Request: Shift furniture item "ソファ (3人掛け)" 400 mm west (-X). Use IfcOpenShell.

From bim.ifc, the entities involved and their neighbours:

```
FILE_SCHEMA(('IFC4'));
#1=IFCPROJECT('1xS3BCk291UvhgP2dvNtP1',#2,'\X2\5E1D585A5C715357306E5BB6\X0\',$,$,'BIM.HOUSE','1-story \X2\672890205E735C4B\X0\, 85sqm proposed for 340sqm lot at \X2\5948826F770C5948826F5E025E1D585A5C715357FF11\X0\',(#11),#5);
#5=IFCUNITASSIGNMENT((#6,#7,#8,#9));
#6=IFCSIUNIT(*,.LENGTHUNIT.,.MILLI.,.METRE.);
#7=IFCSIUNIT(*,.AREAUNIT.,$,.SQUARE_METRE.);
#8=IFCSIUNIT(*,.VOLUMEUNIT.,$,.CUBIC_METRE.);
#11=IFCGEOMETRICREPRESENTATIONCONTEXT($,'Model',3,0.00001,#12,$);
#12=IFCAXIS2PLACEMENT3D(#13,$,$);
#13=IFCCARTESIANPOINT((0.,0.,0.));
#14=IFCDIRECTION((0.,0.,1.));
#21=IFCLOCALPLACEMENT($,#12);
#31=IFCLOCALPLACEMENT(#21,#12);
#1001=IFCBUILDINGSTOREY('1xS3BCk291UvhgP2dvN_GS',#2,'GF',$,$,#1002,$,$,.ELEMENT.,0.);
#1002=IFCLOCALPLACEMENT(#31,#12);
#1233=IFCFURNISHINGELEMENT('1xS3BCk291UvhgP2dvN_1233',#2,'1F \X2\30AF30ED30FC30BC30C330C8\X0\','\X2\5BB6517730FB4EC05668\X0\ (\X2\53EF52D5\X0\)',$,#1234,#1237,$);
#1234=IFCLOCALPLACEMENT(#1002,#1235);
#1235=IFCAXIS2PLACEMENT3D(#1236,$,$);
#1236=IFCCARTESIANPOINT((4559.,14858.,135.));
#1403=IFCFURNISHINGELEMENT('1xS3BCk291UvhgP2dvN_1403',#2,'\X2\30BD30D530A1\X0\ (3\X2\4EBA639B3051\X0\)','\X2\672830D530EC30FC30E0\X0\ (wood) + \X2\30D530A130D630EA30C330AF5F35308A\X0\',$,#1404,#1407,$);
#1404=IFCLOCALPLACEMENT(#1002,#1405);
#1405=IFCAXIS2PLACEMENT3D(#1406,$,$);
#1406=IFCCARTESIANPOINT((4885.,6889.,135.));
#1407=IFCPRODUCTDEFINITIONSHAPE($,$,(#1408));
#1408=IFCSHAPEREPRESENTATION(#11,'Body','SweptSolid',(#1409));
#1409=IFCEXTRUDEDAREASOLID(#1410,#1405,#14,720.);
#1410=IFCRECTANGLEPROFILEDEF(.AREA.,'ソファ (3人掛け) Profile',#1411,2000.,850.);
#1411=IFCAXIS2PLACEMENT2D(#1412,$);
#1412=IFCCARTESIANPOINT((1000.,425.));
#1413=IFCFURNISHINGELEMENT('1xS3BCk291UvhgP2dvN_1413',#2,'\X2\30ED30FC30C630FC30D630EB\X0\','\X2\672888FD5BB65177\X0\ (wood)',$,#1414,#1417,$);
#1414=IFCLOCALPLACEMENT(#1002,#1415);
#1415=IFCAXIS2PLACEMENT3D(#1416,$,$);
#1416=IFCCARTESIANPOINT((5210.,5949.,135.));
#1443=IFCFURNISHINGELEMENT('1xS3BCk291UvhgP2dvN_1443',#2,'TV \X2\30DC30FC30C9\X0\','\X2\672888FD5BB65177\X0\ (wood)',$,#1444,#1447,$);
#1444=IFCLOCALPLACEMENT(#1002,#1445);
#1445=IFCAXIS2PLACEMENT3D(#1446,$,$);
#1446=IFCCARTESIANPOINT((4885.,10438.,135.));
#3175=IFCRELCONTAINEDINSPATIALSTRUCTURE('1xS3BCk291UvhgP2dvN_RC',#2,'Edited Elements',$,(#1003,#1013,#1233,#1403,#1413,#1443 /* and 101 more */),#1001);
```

```python
import ifcopenshell
import ifcopenshell.api.geometry
import ifcopenshell.util.placement
import ifcopenshell.util.unit

model = ifcopenshell.open("bim.ifc")
unit_scale = ifcopenshell.util.unit.calculate_unit_scale(model)

item = model.by_id(1403)
matrix = ifcopenshell.util.placement.get_local_placement(item.ObjectPlacement)
matrix[0, 3] -= 0.4 / unit_scale
ifcopenshell.api.geometry.edit_object_placement(model, product=item, matrix=matrix, is_si=False)

print(ifcopenshell.util.placement.get_local_placement(item.ObjectPlacement).round(3) + 0.0)

model.write("bim_updated.ifc")
```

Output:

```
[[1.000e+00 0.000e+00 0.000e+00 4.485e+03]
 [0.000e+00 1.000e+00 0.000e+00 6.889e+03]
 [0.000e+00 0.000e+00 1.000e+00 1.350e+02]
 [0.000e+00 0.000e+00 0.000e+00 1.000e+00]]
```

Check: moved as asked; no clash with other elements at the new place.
